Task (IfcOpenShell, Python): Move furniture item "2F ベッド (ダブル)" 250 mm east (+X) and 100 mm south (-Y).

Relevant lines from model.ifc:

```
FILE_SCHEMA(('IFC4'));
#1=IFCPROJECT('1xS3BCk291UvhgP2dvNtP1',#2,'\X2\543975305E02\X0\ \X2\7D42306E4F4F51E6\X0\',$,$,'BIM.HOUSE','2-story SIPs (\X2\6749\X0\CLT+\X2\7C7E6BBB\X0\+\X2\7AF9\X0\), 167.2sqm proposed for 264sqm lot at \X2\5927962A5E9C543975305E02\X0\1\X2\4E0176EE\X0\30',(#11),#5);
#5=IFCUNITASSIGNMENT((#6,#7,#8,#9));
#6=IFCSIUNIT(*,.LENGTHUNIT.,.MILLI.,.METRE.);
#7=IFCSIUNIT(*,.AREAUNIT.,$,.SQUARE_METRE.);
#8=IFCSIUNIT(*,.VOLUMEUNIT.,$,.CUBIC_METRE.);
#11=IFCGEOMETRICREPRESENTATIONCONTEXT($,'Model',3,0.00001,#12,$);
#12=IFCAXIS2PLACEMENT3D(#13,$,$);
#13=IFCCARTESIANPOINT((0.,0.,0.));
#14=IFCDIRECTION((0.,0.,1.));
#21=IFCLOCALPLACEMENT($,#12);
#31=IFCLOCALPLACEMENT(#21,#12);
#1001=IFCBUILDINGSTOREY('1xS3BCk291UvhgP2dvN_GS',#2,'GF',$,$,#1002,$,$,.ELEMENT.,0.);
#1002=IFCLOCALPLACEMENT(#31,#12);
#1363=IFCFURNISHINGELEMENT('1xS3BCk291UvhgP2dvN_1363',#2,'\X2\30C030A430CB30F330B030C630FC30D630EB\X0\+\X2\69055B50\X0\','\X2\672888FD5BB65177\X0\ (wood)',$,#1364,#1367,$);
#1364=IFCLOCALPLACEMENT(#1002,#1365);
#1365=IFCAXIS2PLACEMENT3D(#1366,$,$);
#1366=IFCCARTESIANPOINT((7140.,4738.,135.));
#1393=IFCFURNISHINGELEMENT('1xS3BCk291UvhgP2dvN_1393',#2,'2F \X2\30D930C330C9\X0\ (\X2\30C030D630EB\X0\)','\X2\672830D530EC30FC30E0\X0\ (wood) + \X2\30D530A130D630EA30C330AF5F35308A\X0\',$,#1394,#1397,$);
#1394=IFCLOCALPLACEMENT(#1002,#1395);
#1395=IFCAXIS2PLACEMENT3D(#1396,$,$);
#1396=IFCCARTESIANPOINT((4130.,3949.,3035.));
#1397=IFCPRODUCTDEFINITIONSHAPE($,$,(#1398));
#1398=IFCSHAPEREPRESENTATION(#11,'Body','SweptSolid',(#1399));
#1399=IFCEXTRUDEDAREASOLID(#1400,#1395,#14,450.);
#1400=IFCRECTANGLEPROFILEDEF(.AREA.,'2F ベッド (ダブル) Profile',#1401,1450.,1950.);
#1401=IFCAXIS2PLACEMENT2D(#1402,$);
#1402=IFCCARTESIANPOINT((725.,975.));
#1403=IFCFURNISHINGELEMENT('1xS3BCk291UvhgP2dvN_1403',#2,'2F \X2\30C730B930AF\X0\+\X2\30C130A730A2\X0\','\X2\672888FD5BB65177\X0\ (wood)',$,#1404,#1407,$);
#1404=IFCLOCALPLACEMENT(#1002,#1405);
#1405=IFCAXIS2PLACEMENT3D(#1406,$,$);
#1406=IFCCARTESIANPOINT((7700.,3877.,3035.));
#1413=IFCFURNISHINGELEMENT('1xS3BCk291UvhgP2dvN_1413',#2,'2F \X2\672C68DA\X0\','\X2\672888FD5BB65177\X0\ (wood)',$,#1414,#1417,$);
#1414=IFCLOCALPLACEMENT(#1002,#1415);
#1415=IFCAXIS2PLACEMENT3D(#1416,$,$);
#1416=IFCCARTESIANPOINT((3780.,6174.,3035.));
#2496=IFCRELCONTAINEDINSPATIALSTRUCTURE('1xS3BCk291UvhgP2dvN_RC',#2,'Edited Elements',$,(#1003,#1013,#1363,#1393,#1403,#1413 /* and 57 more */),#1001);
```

```python
import ifcopenshell
import ifcopenshell.api.geometry
import ifcopenshell.util.placement
import ifcopenshell.util.unit

model = ifcopenshell.open("model.ifc")
unit_scale = ifcopenshell.util.unit.calculate_unit_scale(model)

item = model.by_guid("1xS3BCk291UvhgP2dvN_1393")
matrix = ifcopenshell.util.placement.get_local_placement(item.ObjectPlacement)
matrix[0, 3] += 0.25 / unit_scale
matrix[1, 3] -= 0.1 / unit_scale
ifcopenshell.api.geometry.edit_object_placement(model, product=item, matrix=matrix, is_si=False)

print(ifcopenshell.util.placement.get_local_placement(item.ObjectPlacement).round(3) + 0.0)

model.write("model_v2.ifc")
```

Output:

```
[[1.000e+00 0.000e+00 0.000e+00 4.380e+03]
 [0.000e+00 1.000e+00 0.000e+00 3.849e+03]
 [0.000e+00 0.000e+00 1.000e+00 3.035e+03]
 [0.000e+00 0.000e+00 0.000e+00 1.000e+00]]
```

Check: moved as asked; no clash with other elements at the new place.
